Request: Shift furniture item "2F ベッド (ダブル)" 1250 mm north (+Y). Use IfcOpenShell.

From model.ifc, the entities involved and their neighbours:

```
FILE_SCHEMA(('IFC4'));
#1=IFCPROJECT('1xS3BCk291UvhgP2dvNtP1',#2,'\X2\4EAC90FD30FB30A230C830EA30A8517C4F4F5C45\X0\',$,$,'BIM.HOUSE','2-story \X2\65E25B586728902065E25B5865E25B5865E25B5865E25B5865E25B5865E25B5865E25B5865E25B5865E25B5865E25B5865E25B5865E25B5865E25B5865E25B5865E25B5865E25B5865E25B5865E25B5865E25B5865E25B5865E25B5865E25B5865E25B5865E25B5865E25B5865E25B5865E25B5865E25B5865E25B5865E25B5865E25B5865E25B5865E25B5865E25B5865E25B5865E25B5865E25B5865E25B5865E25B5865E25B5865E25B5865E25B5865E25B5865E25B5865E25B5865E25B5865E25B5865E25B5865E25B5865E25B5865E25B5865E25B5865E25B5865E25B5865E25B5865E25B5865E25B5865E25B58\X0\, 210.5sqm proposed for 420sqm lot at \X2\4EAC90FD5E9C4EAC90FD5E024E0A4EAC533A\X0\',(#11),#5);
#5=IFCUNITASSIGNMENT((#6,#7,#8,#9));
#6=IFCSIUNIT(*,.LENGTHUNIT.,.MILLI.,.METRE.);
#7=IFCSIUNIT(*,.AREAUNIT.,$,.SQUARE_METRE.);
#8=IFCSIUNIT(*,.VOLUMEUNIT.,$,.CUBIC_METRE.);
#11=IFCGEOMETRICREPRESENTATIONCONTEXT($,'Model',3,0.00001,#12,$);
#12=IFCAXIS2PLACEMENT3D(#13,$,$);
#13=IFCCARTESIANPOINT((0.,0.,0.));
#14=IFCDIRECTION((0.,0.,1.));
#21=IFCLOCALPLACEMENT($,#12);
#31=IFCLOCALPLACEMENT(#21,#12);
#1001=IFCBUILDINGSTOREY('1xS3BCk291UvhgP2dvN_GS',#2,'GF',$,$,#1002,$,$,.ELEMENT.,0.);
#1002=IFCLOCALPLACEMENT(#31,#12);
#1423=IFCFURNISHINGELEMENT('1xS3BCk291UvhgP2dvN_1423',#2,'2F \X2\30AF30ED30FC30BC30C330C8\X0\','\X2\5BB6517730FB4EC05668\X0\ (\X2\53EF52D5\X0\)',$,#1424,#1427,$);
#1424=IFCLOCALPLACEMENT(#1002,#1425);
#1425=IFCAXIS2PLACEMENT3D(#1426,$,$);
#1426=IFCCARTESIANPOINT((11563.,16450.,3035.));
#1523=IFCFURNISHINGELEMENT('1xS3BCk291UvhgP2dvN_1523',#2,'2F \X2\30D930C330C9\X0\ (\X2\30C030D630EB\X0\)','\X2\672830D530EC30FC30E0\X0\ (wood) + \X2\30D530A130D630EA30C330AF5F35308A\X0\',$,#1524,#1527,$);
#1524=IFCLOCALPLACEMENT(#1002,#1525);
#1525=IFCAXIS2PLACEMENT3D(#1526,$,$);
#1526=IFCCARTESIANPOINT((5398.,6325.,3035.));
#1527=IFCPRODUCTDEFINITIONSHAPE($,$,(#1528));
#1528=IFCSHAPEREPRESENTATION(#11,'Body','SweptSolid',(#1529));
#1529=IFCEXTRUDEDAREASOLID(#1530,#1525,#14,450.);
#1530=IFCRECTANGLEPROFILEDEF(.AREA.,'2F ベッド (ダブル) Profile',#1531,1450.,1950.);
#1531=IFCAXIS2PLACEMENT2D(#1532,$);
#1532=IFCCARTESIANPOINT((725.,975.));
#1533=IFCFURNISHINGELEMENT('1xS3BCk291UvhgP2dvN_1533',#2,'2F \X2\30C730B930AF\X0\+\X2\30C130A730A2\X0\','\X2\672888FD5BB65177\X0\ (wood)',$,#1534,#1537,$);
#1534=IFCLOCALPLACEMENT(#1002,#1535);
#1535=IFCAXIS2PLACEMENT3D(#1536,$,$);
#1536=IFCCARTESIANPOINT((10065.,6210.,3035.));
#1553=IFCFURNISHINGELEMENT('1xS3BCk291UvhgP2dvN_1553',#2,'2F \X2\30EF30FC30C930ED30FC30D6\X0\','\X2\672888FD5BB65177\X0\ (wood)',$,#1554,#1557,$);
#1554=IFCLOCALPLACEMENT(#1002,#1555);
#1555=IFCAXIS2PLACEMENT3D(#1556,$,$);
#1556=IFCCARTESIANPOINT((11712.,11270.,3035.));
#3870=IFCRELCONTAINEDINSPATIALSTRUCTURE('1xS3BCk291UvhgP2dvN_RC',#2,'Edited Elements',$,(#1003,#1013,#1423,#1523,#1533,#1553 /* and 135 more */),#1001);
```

```python
import ifcopenshell
import ifcopenshell.api.geometry
import ifcopenshell.util.placement
import ifcopenshell.util.unit

model = ifcopenshell.open("model.ifc")
unit_scale = ifcopenshell.util.unit.calculate_unit_scale(model)

item = model.by_guid("1xS3BCk291UvhgP2dvN_1523")
matrix = ifcopenshell.util.placement.get_local_placement(item.ObjectPlacement)
matrix[1, 3] += 1.25 / unit_scale
ifcopenshell.api.geometry.edit_object_placement(model, product=item, matrix=matrix, is_si=False)

print(ifcopenshell.util.placement.get_local_placement(item.ObjectPlacement).round(3) + 0.0)

model.write("model_rev.ifc")
```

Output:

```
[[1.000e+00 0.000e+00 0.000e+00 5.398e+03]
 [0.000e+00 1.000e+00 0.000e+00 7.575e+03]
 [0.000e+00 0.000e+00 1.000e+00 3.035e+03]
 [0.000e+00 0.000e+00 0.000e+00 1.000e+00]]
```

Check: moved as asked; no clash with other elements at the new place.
